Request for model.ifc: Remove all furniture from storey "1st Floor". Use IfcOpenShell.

First a look at what the model holds.

```python
import ifcopenshell
import ifcopenshell.util.element

model = ifcopenshell.open("model.ifc")
print(model.schema)
storey = next(s for s in model.by_type("IfcBuildingStorey") if s.Name == "1st Floor")
furniture = [e for e in ifcopenshell.util.element.get_decomposition(storey) if e.is_a("IfcFurnishingElement")]
seen = {}
for e in furniture:
    element_type = ifcopenshell.util.element.get_type(e)
    name = element_type.Name if element_type not in (None, e) else None
    seen[name] = seen.get(name, 0) + 1
for name, count in sorted(seen.items(), key=str):
    print(count, "x", name)
```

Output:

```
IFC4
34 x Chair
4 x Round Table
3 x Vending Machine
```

```python
import ifcopenshell
import ifcopenshell.api.root
import ifcopenshell.util.element

model = ifcopenshell.open("model.ifc")

storey = next(s for s in model.by_type("IfcBuildingStorey") if s.Name == "1st Floor")
furniture = [e for e in ifcopenshell.util.element.get_decomposition(storey) if e.is_a("IfcFurnishingElement")]

for e in furniture:
    ifcopenshell.api.root.remove_product(model, product=e)
print(len(furniture), "removed")

model.write("model_v2.ifc")
```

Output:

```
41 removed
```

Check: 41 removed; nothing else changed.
